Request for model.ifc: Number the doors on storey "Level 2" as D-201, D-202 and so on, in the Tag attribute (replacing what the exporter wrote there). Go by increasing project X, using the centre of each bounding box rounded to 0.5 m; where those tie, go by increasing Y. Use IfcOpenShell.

First a look at what the model holds.

```python
import ifcopenshell
import ifcopenshell.util.element
import ifcopenshell.util.placement

model = ifcopenshell.open("model.ifc")
print(model.schema)
storey = next(s for s in model.by_type("IfcBuildingStorey") if s.Name == "Level 2")
doors = [e for e in ifcopenshell.util.element.get_decomposition(storey) if e.is_a("IfcDoor")]
for e in sorted(doors, key=lambda e: e.id()):
    origin = ifcopenshell.util.placement.get_local_placement(e.ObjectPlacement)[:3, 3]
    print(e.id(), e.Tag, e.Name, origin.round(2) + 0.0, sep=" | ")
```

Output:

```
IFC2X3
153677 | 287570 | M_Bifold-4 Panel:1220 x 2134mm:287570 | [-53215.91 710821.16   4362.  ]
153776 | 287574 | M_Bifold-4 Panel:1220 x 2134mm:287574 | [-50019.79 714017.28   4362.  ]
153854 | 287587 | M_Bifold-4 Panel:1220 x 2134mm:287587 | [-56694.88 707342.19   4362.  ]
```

```python
import ifcopenshell
import ifcopenshell.geom
import ifcopenshell.util.element
import ifcopenshell.util.shape

model = ifcopenshell.open("model.ifc")
settings = ifcopenshell.geom.settings()
settings.set("use-world-coords", True)


def centre(element):
    shape = ifcopenshell.geom.create_shape(settings, element)
    return ifcopenshell.util.shape.get_bbox_centroid(shape.geometry)


storey = next(s for s in model.by_type("IfcBuildingStorey") if s.Name == "Level 2")
doors = [e for e in ifcopenshell.util.element.get_decomposition(storey) if e.is_a("IfcDoor")]

# Insertion points can sit at a corner or the storey origin, so sort by the geometry (in metres).
centres = {e: centre(e) for e in doors}
doors.sort(key=lambda e: (round(centres[e][0] / 0.5), centres[e][1]))

for i, e in enumerate(doors, start=1):
    number = f"D-2{i:02d}"
    e.Tag = number
    print(e.id(), number)

model.write("model_updated.ifc")
```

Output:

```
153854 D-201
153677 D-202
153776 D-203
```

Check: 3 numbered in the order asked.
